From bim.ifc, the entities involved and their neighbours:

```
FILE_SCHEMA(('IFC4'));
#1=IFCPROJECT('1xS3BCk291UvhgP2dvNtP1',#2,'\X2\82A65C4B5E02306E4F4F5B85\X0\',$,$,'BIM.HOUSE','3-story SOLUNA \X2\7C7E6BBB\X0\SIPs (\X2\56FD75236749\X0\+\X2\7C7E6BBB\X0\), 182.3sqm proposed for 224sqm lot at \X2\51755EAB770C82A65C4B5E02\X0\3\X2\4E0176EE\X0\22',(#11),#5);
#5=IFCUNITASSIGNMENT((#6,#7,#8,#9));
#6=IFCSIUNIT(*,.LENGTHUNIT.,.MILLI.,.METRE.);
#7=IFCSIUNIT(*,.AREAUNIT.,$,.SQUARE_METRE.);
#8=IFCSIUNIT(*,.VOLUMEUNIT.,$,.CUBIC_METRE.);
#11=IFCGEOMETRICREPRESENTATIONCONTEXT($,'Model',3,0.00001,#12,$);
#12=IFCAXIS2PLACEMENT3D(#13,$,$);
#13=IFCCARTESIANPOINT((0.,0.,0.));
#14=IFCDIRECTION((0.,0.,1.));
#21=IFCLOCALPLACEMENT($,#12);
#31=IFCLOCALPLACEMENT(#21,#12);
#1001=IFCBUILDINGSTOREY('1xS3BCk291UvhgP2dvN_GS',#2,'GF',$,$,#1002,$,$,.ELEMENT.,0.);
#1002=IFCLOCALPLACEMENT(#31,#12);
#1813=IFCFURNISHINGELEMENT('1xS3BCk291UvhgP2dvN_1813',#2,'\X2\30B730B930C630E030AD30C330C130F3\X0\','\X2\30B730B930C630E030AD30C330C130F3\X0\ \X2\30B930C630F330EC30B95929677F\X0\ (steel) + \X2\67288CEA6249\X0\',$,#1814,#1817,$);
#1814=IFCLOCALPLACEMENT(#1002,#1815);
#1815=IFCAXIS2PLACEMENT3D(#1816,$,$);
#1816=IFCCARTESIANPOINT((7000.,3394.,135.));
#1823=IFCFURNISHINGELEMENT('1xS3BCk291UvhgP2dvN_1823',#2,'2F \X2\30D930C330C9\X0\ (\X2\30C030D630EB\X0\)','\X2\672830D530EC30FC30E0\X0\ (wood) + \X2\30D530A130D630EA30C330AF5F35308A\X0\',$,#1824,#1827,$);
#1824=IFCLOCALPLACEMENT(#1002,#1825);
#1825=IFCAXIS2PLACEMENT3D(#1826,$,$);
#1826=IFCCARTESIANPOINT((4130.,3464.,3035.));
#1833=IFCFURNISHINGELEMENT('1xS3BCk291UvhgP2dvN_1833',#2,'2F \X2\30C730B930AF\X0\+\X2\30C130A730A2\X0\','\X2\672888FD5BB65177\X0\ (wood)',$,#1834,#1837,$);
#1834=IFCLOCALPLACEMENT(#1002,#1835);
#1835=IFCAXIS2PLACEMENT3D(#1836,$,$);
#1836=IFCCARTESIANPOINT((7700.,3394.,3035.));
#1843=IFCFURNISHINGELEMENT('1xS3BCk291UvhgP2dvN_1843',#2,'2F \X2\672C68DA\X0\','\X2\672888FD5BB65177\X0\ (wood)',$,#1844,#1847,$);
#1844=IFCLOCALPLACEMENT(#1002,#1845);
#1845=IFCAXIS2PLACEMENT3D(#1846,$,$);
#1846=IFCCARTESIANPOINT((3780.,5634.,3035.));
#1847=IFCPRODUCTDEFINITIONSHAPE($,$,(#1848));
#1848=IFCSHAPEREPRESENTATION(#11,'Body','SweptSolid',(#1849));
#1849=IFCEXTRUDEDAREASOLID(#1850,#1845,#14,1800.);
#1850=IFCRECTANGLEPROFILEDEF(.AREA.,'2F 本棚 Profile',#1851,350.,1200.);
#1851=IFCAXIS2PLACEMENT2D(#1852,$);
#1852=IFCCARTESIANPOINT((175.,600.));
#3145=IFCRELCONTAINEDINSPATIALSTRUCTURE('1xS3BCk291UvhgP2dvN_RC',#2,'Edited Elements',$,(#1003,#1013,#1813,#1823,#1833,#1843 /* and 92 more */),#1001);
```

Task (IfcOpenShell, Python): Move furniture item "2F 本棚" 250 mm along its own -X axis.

```python
import ifcopenshell
import ifcopenshell.api.geometry
import ifcopenshell.util.placement
import ifcopenshell.util.unit

model = ifcopenshell.open("bim.ifc")
unit_scale = ifcopenshell.util.unit.calculate_unit_scale(model)

item = model.by_guid("1xS3BCk291UvhgP2dvN_1843")
matrix = ifcopenshell.util.placement.get_local_placement(item.ObjectPlacement)
matrix[:3, 3] -= matrix[:3, 0] * 0.25 / unit_scale
ifcopenshell.api.geometry.edit_object_placement(model, product=item, matrix=matrix, is_si=False)

print(ifcopenshell.util.placement.get_local_placement(item.ObjectPlacement).round(3) + 0.0)

model.write("bim-out.ifc")
```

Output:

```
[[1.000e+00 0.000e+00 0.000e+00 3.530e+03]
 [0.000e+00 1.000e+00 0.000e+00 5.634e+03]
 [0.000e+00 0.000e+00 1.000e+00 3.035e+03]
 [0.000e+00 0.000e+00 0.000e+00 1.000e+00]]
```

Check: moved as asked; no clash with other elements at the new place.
